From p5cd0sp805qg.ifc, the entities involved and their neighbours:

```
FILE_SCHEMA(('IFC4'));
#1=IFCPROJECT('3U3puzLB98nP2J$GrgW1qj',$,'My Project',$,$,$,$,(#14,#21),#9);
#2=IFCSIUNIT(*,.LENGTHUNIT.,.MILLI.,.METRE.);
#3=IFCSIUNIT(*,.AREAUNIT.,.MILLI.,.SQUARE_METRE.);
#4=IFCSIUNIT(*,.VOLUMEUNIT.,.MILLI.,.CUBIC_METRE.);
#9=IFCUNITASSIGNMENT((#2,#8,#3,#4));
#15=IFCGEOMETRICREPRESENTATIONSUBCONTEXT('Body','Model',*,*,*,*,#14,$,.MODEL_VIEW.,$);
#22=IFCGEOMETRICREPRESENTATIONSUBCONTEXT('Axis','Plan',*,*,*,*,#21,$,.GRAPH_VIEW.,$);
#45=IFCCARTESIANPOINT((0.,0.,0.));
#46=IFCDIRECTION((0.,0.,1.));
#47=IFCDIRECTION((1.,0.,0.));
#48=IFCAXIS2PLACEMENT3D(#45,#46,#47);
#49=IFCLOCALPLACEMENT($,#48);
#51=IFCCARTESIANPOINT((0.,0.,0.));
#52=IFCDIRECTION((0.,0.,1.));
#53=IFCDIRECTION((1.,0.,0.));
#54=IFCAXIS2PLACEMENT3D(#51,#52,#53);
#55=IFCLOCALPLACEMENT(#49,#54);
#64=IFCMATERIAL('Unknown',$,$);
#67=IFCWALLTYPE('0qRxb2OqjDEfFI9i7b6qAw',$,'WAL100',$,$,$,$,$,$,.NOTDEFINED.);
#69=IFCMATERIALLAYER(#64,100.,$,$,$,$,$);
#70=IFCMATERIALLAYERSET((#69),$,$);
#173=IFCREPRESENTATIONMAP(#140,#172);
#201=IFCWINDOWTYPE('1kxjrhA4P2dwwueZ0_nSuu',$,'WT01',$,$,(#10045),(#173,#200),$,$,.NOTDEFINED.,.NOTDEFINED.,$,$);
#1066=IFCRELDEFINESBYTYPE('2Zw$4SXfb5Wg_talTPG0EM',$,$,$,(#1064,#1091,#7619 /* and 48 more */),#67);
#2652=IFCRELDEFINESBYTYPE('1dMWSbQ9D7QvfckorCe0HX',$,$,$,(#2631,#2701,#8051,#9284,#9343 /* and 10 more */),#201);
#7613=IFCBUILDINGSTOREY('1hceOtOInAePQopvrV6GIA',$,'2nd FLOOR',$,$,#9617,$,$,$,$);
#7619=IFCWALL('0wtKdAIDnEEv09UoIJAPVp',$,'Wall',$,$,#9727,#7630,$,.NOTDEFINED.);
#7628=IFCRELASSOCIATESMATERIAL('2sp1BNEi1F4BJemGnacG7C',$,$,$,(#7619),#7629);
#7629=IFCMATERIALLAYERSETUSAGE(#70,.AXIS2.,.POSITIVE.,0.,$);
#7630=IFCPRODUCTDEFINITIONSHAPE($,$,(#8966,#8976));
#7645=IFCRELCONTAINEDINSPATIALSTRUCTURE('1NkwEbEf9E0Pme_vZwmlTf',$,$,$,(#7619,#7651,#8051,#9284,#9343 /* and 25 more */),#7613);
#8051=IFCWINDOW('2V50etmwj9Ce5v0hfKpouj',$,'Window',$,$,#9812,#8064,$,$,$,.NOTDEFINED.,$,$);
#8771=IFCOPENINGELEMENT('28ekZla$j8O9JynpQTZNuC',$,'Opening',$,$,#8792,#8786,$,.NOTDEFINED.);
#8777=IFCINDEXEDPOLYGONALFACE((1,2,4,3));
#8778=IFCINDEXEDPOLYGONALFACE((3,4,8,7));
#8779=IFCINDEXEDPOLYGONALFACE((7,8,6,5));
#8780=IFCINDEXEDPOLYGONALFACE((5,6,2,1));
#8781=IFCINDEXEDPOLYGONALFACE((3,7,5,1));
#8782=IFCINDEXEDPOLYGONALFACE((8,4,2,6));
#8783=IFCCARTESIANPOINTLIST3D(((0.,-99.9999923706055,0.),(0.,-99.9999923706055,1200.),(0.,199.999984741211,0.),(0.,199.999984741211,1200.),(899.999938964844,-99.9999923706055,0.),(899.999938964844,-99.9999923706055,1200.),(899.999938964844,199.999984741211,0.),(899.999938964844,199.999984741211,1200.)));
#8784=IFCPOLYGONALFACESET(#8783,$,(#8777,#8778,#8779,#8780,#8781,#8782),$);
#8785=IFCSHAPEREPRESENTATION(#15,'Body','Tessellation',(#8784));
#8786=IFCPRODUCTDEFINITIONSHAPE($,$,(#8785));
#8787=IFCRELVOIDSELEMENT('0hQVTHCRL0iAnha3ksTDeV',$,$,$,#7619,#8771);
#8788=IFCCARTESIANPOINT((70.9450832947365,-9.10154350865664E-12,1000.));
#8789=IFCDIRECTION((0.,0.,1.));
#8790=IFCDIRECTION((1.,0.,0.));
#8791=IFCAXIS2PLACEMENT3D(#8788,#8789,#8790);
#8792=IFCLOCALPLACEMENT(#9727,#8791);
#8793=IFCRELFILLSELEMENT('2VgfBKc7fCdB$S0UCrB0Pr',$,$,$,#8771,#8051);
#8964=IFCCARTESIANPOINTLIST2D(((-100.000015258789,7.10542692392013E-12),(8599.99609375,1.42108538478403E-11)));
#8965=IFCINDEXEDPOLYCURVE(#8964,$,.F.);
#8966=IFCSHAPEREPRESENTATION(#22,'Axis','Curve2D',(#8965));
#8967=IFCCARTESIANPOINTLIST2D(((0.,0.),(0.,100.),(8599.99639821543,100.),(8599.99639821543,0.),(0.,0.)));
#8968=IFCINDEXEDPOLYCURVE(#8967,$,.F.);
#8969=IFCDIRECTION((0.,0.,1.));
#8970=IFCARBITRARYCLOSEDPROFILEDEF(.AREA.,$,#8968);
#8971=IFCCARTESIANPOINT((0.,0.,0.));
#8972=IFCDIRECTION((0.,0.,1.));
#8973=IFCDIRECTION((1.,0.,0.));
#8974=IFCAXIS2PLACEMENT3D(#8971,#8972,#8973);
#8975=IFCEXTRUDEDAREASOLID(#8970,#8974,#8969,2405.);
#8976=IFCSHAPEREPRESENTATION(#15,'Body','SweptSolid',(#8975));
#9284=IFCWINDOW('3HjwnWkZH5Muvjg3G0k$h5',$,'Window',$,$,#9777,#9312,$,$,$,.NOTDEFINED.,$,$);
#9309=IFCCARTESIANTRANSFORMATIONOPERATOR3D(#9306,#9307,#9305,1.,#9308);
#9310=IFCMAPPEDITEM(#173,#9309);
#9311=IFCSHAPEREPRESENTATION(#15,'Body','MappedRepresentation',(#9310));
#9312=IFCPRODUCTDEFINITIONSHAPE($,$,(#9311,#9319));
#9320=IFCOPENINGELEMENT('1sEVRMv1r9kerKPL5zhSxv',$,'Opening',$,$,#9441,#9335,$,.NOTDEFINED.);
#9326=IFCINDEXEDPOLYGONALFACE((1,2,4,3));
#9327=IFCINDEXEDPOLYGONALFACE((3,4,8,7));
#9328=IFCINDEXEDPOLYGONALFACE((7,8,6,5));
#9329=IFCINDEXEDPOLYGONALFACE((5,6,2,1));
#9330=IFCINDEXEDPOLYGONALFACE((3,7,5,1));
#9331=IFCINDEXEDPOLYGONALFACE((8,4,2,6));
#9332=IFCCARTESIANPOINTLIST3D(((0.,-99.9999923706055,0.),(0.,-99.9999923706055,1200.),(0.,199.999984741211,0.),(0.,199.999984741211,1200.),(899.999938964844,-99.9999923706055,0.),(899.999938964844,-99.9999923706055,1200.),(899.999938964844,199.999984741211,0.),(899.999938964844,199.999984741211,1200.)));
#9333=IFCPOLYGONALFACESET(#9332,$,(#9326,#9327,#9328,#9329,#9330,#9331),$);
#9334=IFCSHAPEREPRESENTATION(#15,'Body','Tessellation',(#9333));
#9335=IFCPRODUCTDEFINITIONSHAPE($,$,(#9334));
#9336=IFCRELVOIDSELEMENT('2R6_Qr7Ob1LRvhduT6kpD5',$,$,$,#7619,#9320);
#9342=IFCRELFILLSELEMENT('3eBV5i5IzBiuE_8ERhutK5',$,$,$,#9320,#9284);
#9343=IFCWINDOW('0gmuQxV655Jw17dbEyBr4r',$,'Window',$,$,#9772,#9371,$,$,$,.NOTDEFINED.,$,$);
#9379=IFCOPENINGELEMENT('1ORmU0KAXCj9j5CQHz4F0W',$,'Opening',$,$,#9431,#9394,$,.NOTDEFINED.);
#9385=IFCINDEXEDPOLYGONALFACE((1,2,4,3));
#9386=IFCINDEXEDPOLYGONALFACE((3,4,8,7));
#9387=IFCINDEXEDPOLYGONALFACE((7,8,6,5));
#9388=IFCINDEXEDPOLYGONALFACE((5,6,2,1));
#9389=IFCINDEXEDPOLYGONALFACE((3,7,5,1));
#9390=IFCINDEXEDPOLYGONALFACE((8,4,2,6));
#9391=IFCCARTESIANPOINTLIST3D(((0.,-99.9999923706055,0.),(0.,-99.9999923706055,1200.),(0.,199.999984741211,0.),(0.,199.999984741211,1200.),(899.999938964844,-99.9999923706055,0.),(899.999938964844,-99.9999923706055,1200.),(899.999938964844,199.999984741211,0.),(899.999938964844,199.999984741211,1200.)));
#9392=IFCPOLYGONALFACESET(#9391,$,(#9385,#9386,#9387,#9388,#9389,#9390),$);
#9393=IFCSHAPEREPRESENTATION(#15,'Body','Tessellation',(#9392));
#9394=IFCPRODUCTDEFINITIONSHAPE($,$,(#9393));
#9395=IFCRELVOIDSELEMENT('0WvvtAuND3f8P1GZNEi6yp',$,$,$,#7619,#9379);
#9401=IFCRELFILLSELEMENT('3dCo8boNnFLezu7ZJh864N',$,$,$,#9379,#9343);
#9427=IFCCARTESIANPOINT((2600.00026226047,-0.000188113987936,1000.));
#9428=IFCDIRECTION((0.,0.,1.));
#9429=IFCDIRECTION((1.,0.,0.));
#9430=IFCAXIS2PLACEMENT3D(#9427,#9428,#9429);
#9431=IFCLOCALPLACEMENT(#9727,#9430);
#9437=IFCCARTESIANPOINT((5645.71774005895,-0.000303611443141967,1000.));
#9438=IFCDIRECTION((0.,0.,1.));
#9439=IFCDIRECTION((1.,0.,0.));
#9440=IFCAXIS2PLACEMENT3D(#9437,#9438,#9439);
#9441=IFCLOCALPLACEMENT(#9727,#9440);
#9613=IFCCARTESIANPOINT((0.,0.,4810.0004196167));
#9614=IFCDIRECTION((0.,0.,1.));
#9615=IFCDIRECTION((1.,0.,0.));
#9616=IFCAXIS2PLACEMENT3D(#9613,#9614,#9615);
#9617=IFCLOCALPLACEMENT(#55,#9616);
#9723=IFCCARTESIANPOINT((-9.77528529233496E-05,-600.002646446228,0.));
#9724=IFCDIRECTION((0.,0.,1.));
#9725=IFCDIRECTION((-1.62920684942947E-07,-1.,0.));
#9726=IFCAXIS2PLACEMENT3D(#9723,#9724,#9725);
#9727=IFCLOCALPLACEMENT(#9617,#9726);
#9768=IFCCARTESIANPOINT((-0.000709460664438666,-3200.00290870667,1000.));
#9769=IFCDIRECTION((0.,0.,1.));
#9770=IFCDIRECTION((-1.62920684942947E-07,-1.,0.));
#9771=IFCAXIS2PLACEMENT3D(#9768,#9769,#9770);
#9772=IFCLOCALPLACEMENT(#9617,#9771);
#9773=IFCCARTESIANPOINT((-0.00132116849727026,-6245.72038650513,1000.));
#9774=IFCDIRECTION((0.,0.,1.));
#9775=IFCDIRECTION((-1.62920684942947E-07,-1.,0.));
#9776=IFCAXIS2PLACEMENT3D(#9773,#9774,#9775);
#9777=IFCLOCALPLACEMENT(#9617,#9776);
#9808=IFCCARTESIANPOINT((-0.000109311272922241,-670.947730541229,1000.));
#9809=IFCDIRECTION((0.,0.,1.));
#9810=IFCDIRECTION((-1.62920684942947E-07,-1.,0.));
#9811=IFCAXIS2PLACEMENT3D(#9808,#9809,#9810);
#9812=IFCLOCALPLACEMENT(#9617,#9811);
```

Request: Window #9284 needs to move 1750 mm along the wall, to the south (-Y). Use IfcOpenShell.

```python
import ifcopenshell
import ifcopenshell.api.geometry
import ifcopenshell.util.placement

model = ifcopenshell.open("p5cd0sp805qg.ifc")

window = model.by_guid("3HjwnWkZH5Muvjg3G0k$h5")
opening = window.FillsVoids[0].RelatingOpeningElement
wall = opening.VoidsElements[0].RelatingBuildingElement

wall_matrix = ifcopenshell.util.placement.get_local_placement(wall.ObjectPlacement)
shift = wall_matrix[:3, 0] * 1750.0
before = ifcopenshell.util.placement.get_local_placement(window.ObjectPlacement)[:3, 3].copy()

# The window is not placed relative to its opening, so move both.
for product in (opening, window):
    matrix = ifcopenshell.util.placement.get_local_placement(product.ObjectPlacement)
    matrix[:3, 3] += shift
    ifcopenshell.api.geometry.edit_object_placement(model, product=product, matrix=matrix, is_si=False)

after = ifcopenshell.util.placement.get_local_placement(window.ObjectPlacement)[:3, 3]
print("window moved by", (after - before).round(3) + 0.0)

model.write("p5cd0sp805qg_v2.ifc")
```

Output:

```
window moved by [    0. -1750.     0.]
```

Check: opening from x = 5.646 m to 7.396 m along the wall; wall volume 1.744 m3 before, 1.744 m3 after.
